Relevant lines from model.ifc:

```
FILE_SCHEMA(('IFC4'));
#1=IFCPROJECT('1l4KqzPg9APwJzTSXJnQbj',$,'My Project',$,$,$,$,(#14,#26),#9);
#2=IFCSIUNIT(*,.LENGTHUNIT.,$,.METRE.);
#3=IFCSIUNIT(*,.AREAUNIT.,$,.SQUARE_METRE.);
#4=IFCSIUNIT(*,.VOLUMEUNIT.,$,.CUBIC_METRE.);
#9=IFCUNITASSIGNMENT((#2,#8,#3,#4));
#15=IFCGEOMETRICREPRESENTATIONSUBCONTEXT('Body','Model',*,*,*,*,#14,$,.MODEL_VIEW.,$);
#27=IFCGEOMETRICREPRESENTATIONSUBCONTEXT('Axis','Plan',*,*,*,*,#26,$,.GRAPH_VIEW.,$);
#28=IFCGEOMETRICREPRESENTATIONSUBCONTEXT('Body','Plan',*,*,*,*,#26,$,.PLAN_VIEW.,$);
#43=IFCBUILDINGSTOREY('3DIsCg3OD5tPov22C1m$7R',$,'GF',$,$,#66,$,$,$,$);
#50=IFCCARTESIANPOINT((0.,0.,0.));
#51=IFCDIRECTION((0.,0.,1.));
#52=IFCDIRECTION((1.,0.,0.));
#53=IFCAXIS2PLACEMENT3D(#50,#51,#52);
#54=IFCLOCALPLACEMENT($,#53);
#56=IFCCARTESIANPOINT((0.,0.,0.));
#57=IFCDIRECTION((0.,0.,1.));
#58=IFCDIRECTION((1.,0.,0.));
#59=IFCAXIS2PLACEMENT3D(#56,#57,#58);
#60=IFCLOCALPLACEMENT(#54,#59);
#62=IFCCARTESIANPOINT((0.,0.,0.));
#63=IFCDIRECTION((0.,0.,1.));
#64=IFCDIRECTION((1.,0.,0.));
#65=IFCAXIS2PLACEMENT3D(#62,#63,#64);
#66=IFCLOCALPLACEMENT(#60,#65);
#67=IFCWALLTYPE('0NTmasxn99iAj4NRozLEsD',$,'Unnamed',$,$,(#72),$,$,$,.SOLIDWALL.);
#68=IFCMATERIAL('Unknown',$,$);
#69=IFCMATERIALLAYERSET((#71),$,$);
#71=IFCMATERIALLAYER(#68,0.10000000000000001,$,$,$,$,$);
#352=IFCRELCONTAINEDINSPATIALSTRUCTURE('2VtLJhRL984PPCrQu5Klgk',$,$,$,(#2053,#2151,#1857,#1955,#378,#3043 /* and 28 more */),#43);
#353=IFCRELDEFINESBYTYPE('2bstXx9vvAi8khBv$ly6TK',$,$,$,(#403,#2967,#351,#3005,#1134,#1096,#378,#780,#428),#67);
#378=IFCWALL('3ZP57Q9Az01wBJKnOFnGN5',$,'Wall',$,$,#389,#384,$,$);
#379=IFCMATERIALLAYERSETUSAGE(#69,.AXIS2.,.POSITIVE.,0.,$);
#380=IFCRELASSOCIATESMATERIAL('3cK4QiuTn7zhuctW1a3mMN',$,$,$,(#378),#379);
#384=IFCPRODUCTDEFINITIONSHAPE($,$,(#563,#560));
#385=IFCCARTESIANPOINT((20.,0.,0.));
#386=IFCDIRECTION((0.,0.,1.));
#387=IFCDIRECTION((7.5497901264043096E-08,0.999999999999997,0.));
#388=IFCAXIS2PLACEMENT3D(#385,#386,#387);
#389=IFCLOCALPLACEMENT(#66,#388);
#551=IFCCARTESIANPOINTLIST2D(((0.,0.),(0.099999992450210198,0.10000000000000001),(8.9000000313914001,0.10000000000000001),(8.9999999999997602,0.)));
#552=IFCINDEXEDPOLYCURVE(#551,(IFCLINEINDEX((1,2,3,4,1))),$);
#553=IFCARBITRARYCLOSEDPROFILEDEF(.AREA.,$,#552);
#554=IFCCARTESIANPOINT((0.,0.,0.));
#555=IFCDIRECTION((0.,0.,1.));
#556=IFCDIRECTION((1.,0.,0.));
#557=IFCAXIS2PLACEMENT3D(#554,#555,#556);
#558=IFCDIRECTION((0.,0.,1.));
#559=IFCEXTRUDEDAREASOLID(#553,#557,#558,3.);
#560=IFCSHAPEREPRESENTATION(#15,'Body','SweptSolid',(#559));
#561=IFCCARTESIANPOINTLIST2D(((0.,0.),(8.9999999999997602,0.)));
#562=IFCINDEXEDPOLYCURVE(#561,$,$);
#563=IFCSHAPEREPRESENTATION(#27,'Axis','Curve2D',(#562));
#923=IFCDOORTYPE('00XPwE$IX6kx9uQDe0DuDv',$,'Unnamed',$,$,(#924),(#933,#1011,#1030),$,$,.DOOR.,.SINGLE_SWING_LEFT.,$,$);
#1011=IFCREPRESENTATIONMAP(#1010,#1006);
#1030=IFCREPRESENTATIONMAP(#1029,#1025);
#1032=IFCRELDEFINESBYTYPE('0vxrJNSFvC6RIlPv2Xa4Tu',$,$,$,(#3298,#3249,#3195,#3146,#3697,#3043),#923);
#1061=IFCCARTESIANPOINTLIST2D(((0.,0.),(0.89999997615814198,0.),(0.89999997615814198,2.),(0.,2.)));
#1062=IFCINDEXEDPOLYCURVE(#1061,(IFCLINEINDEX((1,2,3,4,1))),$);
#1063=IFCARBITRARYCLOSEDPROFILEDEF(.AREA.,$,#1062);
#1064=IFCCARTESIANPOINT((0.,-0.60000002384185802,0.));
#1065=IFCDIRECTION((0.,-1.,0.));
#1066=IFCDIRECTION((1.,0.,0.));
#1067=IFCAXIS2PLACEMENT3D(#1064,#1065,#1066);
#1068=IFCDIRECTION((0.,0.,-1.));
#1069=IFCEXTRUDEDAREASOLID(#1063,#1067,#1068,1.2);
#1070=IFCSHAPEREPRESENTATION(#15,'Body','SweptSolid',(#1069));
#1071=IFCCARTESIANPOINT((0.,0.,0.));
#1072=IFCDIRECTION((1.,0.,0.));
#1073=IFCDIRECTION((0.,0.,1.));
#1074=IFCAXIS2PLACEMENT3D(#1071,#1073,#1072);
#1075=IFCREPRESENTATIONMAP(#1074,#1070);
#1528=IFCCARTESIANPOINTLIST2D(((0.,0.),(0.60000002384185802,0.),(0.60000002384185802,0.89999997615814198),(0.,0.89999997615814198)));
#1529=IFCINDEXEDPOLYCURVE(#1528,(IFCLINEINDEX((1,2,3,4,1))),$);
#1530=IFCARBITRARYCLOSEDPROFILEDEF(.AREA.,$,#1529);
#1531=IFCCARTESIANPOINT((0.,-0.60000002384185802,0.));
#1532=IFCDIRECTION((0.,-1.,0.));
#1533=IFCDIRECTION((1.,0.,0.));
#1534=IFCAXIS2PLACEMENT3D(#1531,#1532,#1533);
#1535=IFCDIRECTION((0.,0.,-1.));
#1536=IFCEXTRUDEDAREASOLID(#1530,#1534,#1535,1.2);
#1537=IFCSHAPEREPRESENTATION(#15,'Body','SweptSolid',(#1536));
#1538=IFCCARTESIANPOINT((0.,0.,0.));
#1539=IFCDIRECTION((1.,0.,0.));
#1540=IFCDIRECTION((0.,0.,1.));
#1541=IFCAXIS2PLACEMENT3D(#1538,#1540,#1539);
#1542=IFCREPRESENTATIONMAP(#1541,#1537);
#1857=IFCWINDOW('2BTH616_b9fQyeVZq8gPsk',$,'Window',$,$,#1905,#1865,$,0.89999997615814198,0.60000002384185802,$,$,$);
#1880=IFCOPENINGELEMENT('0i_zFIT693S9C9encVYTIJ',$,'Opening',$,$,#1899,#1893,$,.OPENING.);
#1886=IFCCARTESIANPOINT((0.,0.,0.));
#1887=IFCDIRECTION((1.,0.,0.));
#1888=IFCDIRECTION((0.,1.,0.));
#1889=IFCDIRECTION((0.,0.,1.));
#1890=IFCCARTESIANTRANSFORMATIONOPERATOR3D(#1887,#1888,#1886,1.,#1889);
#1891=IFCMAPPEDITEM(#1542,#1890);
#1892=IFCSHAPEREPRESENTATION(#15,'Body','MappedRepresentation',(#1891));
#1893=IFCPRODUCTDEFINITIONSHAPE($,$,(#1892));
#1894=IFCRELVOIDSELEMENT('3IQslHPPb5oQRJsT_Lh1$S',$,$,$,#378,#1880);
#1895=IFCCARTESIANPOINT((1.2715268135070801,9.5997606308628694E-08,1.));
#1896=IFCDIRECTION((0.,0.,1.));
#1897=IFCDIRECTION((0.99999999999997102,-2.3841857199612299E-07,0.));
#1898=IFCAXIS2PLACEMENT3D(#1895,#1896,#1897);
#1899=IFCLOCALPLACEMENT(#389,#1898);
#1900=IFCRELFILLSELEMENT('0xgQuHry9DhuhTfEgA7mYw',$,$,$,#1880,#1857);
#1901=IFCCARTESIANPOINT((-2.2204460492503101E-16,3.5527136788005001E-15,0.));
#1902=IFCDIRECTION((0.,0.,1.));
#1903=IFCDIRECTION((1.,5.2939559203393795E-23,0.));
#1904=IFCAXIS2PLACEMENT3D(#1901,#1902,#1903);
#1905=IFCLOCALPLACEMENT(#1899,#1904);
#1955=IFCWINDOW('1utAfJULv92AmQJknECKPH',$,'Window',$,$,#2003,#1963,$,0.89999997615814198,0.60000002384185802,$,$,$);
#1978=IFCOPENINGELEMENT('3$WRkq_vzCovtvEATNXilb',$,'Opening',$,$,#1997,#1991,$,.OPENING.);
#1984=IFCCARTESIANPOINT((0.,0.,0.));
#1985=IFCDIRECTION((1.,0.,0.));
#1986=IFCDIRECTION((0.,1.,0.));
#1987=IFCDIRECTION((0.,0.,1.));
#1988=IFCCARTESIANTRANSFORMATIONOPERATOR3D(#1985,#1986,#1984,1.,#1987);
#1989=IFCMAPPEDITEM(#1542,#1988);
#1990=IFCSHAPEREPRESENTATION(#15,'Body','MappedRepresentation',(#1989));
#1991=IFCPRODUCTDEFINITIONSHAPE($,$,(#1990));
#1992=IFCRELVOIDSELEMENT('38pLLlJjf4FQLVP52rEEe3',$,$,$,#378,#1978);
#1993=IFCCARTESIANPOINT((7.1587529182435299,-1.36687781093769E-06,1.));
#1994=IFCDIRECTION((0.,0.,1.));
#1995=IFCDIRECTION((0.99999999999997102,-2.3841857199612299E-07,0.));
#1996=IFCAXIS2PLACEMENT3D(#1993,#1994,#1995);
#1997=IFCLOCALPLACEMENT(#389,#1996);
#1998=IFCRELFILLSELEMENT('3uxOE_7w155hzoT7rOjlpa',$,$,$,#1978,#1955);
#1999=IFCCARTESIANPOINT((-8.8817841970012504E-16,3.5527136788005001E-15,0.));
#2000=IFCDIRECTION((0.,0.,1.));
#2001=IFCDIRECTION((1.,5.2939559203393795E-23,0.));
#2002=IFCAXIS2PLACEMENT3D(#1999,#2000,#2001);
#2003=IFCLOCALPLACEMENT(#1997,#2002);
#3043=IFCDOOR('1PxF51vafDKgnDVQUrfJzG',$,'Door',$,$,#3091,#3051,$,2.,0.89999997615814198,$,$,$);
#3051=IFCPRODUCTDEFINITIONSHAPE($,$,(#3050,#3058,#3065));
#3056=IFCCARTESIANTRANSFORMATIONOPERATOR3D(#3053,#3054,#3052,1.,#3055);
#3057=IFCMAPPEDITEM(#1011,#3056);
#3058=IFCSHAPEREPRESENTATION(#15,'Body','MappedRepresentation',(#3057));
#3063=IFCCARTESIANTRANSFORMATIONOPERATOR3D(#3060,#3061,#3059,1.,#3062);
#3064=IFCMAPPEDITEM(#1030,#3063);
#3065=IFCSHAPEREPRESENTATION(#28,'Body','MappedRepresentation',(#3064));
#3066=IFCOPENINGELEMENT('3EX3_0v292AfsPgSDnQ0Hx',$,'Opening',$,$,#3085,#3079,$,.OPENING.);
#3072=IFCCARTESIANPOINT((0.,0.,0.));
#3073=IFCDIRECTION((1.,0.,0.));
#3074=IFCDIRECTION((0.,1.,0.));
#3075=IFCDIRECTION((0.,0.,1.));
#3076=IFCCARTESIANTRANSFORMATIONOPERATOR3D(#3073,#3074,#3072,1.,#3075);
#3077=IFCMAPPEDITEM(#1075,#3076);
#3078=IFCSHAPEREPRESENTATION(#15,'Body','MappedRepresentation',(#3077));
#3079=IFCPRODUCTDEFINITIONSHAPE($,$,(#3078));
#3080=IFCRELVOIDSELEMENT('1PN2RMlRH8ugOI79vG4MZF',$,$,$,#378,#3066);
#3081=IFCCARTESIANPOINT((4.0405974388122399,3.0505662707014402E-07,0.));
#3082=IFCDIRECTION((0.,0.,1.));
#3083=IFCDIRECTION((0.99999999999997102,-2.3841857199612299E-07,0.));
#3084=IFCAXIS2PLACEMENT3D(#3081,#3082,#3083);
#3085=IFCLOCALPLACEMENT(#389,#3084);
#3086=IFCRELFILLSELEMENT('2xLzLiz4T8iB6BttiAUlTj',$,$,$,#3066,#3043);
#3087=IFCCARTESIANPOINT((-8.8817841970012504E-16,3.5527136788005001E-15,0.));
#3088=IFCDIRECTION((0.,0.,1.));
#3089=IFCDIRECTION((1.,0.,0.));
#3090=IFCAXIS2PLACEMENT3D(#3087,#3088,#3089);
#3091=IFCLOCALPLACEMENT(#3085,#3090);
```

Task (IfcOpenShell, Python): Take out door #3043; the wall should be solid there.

```python
import ifcopenshell
import ifcopenshell.api.feature
import ifcopenshell.api.root
import ifcopenshell.geom
import ifcopenshell.util.shape

model = ifcopenshell.open("model.ifc")
settings = ifcopenshell.geom.settings()


def volume(element):
    """Net volume in cubic metres, openings subtracted."""
    shape = ifcopenshell.geom.create_shape(settings, element)
    return ifcopenshell.util.shape.get_volume(shape.geometry)


door = model.by_guid("1PxF51vafDKgnDVQUrfJzG")
opening = door.FillsVoids[0].RelatingOpeningElement
wall = opening.VoidsElements[0].RelatingBuildingElement
before = volume(wall)

ifcopenshell.api.root.remove_product(model, product=door)
ifcopenshell.api.feature.remove_feature(model, feature=opening)

after = volume(wall)

print(f"wall volume {before:.3f} -> {after:.3f} m3")

model.write("model_updated.ifc")
```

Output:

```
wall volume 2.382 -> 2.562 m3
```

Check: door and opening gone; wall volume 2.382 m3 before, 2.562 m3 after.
